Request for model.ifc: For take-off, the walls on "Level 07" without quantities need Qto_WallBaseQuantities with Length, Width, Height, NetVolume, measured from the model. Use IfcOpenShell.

First a look at what the model holds.

```python
import ifcopenshell
import ifcopenshell.util.element
import ifcopenshell.util.unit

model = ifcopenshell.open("model.ifc")
print(model.schema)
for unit_type in ("LENGTHUNIT", "AREAUNIT", "VOLUMEUNIT"):
    print(unit_type, ifcopenshell.util.unit.calculate_unit_scale(model, unit_type))
storey = next(s for s in model.by_type("IfcBuildingStorey") if s.Name == "Level 07")
walls = [e for e in ifcopenshell.util.element.get_decomposition(storey) if e.is_a("IfcWall")]
for e in sorted(walls, key=lambda e: e.id()):
    print(e.id(), e.is_a(), e.Name, list(ifcopenshell.util.element.get_psets(e, qtos_only=True)), sep=" | ")
```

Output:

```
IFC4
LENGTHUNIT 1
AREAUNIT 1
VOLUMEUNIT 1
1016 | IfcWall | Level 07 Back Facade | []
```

```python
import ifcopenshell
import ifcopenshell.api.pset
import ifcopenshell.geom
import ifcopenshell.util.element
import ifcopenshell.util.shape
import ifcopenshell.util.unit

model = ifcopenshell.open("model.ifc")
unit_scale = ifcopenshell.util.unit.calculate_unit_scale(model)
volume_scale = ifcopenshell.util.unit.calculate_unit_scale(model, "VOLUMEUNIT")
settings = ifcopenshell.geom.settings()

storey = next(s for s in model.by_type("IfcBuildingStorey") if s.Name == "Level 07")
walls = [e for e in ifcopenshell.util.element.get_decomposition(storey) if e.is_a("IfcWall")]

for e in sorted(walls, key=lambda e: e.id()):
    if ifcopenshell.util.element.get_psets(e, qtos_only=True, should_inherit=False):
        continue
    # Geometry comes back in metres, in the element's own axes.
    shape = ifcopenshell.geom.create_shape(settings, e)
    values = {
        "Length": ifcopenshell.util.shape.get_x(shape.geometry) / unit_scale,
        "Width": ifcopenshell.util.shape.get_y(shape.geometry) / unit_scale,
        "Height": ifcopenshell.util.shape.get_z(shape.geometry) / unit_scale,
        "NetVolume": ifcopenshell.util.shape.get_volume(shape.geometry) / volume_scale,
    }
    qto = ifcopenshell.api.pset.add_qto(model, product=e, name="Qto_WallBaseQuantities")
    ifcopenshell.api.pset.edit_qto(model, qto=qto, properties=values)
    print(e.id(), {k: round(v, 3) for k, v in values.items()})

model.write("model_v2.ifc")
```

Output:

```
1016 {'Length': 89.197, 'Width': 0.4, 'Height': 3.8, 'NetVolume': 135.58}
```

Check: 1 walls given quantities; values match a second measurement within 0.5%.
